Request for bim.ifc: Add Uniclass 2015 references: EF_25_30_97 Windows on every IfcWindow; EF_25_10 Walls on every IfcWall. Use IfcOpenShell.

First a look at what the model holds.

```python
import ifcopenshell

model = ifcopenshell.open("bim.ifc")
print(model.schema)
print("classifications:", [c.Name for c in model.by_type("IfcClassification")])
for ifc_class in ("IfcDoor", "IfcRoof", "IfcStair", "IfcWall", "IfcWindow"):
    print(ifc_class, len(model.by_type(ifc_class)))
```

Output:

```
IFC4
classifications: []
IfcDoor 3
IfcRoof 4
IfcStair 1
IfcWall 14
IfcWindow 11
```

```python
import ifcopenshell
import ifcopenshell.api.classification

model = ifcopenshell.open("bim.ifc")

system = ifcopenshell.api.classification.add_classification(model, classification="Uniclass 2015")

codes = {
    "IfcWindow": ("EF_25_30_97", "Windows"),
    "IfcWall": ("EF_25_10", "Walls"),
}
for ifc_class, (code, name) in codes.items():
    products = model.by_type(ifc_class)
    ifcopenshell.api.classification.add_reference(
        model, products=products, classification=system, identification=code, name=name
    )
    print(code, len(products))

model.write("bim_updated.ifc")
```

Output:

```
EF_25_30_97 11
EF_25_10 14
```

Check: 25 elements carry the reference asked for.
